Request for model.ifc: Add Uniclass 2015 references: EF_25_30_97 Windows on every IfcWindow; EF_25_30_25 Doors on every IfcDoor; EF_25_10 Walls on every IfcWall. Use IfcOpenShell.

First a look at what the model holds.

```python
import ifcopenshell

model = ifcopenshell.open("model.ifc")
print(model.schema)
print("classifications:", [c.Name for c in model.by_type("IfcClassification")])
for ifc_class in ("IfcDoor", "IfcRoof", "IfcStair", "IfcWall", "IfcWindow"):
    print(ifc_class, len(model.by_type(ifc_class)))
```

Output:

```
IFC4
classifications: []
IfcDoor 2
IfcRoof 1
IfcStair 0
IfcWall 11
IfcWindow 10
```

```python
import ifcopenshell
import ifcopenshell.api.classification

model = ifcopenshell.open("model.ifc")

system = ifcopenshell.api.classification.add_classification(model, classification="Uniclass 2015")

codes = {
    "IfcWindow": ("EF_25_30_97", "Windows"),
    "IfcDoor": ("EF_25_30_25", "Doors"),
    "IfcWall": ("EF_25_10", "Walls"),
}
for ifc_class, (code, name) in codes.items():
    products = model.by_type(ifc_class)
    ifcopenshell.api.classification.add_reference(
        model, products=products, classification=system, identification=code, name=name
    )
    print(code, len(products))

model.write("model_v2.ifc")
```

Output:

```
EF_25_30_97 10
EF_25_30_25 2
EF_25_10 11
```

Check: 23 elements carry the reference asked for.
